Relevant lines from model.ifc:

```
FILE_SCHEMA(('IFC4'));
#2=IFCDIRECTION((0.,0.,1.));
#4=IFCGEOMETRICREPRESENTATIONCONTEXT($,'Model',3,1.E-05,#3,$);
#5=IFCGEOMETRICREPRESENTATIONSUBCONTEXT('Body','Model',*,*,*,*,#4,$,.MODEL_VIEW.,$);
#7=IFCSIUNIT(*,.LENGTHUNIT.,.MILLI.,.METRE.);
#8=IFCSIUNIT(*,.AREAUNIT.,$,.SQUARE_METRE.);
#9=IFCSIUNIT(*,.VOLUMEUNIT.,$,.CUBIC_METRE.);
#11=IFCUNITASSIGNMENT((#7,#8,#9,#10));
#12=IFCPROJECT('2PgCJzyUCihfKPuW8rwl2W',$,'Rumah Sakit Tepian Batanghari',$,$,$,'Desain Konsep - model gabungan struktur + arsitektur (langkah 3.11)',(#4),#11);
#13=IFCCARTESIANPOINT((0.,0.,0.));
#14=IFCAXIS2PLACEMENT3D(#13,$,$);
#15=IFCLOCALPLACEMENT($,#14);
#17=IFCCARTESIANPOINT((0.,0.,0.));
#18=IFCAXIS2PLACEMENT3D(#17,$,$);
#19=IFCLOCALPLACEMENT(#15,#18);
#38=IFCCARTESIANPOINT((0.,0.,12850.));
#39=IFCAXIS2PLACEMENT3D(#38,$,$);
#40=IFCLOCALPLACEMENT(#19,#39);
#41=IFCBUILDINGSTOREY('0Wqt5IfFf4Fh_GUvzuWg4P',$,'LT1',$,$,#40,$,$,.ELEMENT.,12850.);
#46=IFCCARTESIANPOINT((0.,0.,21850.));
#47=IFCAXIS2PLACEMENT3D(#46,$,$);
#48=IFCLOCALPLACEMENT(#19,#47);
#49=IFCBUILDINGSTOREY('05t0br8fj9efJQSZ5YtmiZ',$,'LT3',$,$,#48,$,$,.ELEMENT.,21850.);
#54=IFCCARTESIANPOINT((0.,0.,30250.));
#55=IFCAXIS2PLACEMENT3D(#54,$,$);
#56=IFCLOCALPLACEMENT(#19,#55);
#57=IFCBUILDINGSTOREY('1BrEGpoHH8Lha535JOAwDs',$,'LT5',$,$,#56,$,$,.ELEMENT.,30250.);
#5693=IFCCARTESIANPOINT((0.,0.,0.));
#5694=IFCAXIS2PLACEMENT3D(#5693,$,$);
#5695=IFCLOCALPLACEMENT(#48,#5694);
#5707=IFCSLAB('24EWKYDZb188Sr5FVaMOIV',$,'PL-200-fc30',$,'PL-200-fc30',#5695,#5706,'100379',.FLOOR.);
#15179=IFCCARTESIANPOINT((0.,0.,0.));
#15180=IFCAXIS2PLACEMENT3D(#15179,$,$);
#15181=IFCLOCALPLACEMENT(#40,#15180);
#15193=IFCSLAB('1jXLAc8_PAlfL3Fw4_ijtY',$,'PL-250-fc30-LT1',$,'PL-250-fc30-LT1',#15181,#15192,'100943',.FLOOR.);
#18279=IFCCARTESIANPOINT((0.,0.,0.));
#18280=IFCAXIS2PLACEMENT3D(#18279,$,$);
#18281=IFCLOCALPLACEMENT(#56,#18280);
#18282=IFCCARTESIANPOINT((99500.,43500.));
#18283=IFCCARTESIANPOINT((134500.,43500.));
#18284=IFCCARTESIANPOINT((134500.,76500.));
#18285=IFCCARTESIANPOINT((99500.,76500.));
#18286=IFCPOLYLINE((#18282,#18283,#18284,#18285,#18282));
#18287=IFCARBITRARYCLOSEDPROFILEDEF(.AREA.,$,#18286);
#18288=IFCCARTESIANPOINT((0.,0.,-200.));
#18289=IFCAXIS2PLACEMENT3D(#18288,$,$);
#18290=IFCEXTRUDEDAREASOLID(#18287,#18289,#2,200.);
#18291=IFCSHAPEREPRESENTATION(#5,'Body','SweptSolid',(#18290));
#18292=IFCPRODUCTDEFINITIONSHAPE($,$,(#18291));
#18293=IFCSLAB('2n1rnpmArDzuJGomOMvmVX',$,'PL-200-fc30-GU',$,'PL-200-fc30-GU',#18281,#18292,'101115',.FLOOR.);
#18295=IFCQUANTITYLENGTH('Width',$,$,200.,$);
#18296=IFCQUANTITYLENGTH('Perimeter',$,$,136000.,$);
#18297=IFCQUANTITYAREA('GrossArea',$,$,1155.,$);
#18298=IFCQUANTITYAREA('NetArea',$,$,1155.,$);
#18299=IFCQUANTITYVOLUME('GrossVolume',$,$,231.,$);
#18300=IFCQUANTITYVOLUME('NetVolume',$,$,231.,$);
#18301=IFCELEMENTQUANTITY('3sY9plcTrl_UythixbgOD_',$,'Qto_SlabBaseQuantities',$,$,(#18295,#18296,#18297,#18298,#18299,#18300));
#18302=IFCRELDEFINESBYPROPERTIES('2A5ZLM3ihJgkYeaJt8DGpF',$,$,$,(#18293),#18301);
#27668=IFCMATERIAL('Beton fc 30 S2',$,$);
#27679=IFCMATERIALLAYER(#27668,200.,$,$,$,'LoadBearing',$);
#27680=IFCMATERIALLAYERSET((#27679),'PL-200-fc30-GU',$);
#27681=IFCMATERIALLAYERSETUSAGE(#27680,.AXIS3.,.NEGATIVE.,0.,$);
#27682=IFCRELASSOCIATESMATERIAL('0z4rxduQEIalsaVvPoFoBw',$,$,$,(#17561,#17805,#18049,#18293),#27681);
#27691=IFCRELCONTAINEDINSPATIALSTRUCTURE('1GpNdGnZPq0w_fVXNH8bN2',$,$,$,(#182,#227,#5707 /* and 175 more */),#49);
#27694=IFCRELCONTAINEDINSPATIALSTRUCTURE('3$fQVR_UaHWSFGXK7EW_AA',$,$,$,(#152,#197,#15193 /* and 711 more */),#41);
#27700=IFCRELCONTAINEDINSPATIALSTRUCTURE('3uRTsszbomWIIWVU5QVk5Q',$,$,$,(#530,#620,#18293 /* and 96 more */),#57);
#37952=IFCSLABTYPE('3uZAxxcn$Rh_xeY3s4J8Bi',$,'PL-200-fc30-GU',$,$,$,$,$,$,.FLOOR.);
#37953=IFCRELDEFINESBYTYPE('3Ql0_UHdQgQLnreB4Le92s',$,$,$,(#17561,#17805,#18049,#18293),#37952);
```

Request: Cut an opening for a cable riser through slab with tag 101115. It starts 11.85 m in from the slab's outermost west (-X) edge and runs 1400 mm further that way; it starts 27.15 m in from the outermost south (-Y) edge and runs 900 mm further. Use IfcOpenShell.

```python
import numpy as np
import ifcopenshell
import ifcopenshell.api.feature
import ifcopenshell.api.geometry
import ifcopenshell.api.pset
import ifcopenshell.api.root
import ifcopenshell.geom
import ifcopenshell.util.element
import ifcopenshell.util.placement
import ifcopenshell.util.representation
import ifcopenshell.util.shape
import ifcopenshell.util.unit

model = ifcopenshell.open("model.ifc")
unit_scale = ifcopenshell.util.unit.calculate_unit_scale(model)
area_scale = ifcopenshell.util.unit.calculate_unit_scale(model, "AREAUNIT")
volume_scale = ifcopenshell.util.unit.calculate_unit_scale(model, "VOLUMEUNIT")
settings = ifcopenshell.geom.settings()


def volume(element):
    """Net volume in cubic metres, openings subtracted."""
    shape = ifcopenshell.geom.create_shape(settings, element)
    return ifcopenshell.util.shape.get_volume(shape.geometry)


slab = model.by_guid("2n1rnpmArDzuJGomOMvmVX")
before = volume(slab)

# Extent in the slab's own axes, in metres. The edges named are its -X and -Y sides.
slab_shape = ifcopenshell.geom.create_shape(settings, slab)
vertices = ifcopenshell.util.shape.get_vertices(slab_shape.geometry)
x_min, y_min, bottom = vertices.min(axis=0)
top = vertices[:, 2].max()

opening = ifcopenshell.api.root.create_entity(model, ifc_class="IfcOpeningElement", name="Cable riser opening", predefined_type="OPENING")
context = ifcopenshell.util.representation.get_context(model, "Model", "Body", "MODEL_VIEW")
width, depth = 1.4, 0.9
outline = [(0.0, 0.0), (width, 0.0), (width, depth), (0.0, depth), (0.0, 0.0)]
# Overshoot both faces by 50 mm so the cut is clean.
shape = ifcopenshell.api.geometry.add_slab_representation(
    model, context=context, depth=top - bottom + 0.1, polyline=outline
)
ifcopenshell.api.geometry.assign_representation(model, product=opening, representation=shape)

matrix = ifcopenshell.util.placement.get_local_placement(slab.ObjectPlacement)
matrix[:, 3] = matrix @ np.append(np.array([x_min + 11.85, y_min + 27.15, bottom - 0.05]) / unit_scale, 1.0)
ifcopenshell.api.geometry.edit_object_placement(model, product=opening, matrix=matrix, is_si=False)
ifcopenshell.api.feature.add_feature(model, feature=opening, element=slab)

after = volume(slab)

# Update the slab's stored quantities.
qto = model.by_id(ifcopenshell.util.element.get_pset(slab, "Qto_SlabBaseQuantities", should_inherit=False)["id"])
ifcopenshell.api.pset.edit_qto(model, qto=qto, properties={
    "NetArea": after / (top - bottom) / area_scale,
    "NetVolume": after / volume_scale,
})

print(f"slab volume {before:.3f} -> {after:.3f} m3")

model.write("model_rev.ifc")
```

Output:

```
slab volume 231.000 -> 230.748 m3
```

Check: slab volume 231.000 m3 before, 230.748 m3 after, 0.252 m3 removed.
